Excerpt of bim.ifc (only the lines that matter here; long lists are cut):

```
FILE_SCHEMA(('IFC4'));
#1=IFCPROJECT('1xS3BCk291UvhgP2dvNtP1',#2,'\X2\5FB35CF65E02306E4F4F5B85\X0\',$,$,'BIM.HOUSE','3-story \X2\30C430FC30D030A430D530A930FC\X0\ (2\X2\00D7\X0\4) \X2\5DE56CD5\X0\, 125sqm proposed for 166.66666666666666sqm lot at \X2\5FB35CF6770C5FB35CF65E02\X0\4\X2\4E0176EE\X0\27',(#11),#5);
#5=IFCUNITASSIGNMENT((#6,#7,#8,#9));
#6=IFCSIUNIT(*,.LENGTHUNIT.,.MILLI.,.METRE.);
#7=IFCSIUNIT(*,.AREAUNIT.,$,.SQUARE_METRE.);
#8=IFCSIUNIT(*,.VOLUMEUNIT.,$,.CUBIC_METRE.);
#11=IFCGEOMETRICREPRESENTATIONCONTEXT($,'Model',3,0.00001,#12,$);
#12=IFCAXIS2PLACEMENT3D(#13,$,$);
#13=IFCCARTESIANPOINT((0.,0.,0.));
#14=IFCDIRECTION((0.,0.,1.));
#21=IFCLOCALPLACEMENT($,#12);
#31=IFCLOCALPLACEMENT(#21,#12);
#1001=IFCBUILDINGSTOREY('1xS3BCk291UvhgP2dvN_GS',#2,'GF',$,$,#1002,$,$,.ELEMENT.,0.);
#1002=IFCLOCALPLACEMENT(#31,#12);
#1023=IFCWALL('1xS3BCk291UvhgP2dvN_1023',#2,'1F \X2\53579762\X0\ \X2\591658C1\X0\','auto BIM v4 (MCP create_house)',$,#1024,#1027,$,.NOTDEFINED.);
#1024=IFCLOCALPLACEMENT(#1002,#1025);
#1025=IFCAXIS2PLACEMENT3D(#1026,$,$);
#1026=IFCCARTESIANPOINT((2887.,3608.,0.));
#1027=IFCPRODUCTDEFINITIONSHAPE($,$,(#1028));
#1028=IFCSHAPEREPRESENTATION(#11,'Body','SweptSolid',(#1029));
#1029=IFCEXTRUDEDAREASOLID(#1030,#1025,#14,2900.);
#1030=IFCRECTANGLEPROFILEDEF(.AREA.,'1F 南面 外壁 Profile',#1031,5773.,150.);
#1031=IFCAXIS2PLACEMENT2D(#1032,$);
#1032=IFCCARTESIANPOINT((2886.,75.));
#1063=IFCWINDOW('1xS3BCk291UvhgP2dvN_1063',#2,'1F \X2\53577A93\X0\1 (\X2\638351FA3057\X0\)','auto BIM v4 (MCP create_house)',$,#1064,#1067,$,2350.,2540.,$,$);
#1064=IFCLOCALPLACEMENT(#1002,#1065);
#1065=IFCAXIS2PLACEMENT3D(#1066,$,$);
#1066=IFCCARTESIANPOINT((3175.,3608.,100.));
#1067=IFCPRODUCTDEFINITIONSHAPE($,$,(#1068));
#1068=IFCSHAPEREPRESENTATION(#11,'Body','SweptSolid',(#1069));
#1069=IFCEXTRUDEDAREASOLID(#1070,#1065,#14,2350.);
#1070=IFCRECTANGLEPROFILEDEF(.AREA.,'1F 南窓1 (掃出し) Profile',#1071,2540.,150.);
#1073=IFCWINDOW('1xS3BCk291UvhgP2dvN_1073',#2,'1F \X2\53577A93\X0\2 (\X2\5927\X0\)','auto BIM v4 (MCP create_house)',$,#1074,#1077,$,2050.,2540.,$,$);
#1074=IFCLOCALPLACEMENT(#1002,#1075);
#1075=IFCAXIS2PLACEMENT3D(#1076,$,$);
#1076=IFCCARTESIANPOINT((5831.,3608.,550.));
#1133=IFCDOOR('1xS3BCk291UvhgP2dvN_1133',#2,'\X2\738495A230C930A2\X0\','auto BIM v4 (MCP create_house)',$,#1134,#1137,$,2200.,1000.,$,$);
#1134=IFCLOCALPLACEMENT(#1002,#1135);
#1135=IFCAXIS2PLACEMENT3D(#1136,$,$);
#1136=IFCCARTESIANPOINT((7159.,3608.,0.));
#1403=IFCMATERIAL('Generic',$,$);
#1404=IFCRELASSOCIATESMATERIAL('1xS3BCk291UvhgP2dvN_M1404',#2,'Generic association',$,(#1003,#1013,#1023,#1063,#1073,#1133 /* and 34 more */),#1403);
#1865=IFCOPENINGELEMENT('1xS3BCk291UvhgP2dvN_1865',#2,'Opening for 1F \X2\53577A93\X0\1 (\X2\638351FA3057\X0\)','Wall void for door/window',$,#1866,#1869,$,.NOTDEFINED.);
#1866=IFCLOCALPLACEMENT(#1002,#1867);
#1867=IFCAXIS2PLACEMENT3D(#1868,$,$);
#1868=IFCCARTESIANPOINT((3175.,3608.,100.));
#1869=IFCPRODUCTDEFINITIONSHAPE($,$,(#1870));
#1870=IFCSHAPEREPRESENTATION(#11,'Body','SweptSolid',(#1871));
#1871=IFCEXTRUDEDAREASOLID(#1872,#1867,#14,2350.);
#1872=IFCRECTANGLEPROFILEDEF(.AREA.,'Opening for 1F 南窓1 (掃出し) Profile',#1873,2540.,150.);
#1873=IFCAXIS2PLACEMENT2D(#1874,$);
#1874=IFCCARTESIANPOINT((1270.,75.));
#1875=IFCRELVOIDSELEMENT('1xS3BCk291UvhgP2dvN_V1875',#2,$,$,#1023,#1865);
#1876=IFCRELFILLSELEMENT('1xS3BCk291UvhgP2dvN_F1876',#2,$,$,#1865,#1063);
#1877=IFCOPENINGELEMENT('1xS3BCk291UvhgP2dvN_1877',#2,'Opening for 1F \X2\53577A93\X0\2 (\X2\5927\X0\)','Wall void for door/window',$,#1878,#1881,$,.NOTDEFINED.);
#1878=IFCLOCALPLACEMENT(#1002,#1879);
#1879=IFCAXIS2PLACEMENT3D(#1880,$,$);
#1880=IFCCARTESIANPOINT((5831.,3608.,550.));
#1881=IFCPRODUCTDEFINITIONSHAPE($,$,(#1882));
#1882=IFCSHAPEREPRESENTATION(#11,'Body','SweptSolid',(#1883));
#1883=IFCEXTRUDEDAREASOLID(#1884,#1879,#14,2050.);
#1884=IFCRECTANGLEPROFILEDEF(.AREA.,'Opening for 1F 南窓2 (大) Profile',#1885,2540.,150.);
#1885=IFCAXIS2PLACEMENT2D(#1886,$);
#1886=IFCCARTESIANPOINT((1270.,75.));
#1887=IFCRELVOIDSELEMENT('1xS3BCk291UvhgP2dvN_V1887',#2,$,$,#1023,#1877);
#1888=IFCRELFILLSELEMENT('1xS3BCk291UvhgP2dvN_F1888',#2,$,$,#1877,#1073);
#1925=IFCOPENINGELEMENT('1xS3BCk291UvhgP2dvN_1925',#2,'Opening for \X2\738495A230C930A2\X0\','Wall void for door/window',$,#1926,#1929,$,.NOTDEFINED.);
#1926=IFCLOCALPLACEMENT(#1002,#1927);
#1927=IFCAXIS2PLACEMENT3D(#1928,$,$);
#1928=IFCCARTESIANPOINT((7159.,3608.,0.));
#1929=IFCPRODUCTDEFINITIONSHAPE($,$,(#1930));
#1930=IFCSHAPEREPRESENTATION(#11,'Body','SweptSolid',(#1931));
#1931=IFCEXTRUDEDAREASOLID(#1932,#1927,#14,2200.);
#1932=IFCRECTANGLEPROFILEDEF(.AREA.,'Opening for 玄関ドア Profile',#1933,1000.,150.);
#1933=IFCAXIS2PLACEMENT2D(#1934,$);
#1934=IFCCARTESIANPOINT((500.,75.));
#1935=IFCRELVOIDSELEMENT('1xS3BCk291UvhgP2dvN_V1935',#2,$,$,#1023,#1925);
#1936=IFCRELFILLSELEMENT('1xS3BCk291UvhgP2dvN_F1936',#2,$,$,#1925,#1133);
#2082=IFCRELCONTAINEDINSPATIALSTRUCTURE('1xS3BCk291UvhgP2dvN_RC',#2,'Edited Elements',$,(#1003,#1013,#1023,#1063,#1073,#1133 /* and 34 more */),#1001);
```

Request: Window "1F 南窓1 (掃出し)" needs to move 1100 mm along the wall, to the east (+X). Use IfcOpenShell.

```python
import ifcopenshell
import ifcopenshell.api.geometry
import ifcopenshell.util.placement
import ifcopenshell.util.unit

model = ifcopenshell.open("bim.ifc")
unit_scale = ifcopenshell.util.unit.calculate_unit_scale(model)

window = model.by_id(1063)
opening = window.FillsVoids[0].RelatingOpeningElement
wall = opening.VoidsElements[0].RelatingBuildingElement

wall_matrix = ifcopenshell.util.placement.get_local_placement(wall.ObjectPlacement)
shift = wall_matrix[:3, 0] * 1.1 / unit_scale
before = ifcopenshell.util.placement.get_local_placement(window.ObjectPlacement)[:3, 3].copy()

# The window is not placed relative to its opening, so move both.
for product in (opening, window):
    matrix = ifcopenshell.util.placement.get_local_placement(product.ObjectPlacement)
    matrix[:3, 3] += shift
    ifcopenshell.api.geometry.edit_object_placement(model, product=product, matrix=matrix, is_si=False)

after = ifcopenshell.util.placement.get_local_placement(window.ObjectPlacement)[:3, 3]
print("window moved by", (after - before).round(3) + 0.0)

model.write("bim_rev.ifc")
```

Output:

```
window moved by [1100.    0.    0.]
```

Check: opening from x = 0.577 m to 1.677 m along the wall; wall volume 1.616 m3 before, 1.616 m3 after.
